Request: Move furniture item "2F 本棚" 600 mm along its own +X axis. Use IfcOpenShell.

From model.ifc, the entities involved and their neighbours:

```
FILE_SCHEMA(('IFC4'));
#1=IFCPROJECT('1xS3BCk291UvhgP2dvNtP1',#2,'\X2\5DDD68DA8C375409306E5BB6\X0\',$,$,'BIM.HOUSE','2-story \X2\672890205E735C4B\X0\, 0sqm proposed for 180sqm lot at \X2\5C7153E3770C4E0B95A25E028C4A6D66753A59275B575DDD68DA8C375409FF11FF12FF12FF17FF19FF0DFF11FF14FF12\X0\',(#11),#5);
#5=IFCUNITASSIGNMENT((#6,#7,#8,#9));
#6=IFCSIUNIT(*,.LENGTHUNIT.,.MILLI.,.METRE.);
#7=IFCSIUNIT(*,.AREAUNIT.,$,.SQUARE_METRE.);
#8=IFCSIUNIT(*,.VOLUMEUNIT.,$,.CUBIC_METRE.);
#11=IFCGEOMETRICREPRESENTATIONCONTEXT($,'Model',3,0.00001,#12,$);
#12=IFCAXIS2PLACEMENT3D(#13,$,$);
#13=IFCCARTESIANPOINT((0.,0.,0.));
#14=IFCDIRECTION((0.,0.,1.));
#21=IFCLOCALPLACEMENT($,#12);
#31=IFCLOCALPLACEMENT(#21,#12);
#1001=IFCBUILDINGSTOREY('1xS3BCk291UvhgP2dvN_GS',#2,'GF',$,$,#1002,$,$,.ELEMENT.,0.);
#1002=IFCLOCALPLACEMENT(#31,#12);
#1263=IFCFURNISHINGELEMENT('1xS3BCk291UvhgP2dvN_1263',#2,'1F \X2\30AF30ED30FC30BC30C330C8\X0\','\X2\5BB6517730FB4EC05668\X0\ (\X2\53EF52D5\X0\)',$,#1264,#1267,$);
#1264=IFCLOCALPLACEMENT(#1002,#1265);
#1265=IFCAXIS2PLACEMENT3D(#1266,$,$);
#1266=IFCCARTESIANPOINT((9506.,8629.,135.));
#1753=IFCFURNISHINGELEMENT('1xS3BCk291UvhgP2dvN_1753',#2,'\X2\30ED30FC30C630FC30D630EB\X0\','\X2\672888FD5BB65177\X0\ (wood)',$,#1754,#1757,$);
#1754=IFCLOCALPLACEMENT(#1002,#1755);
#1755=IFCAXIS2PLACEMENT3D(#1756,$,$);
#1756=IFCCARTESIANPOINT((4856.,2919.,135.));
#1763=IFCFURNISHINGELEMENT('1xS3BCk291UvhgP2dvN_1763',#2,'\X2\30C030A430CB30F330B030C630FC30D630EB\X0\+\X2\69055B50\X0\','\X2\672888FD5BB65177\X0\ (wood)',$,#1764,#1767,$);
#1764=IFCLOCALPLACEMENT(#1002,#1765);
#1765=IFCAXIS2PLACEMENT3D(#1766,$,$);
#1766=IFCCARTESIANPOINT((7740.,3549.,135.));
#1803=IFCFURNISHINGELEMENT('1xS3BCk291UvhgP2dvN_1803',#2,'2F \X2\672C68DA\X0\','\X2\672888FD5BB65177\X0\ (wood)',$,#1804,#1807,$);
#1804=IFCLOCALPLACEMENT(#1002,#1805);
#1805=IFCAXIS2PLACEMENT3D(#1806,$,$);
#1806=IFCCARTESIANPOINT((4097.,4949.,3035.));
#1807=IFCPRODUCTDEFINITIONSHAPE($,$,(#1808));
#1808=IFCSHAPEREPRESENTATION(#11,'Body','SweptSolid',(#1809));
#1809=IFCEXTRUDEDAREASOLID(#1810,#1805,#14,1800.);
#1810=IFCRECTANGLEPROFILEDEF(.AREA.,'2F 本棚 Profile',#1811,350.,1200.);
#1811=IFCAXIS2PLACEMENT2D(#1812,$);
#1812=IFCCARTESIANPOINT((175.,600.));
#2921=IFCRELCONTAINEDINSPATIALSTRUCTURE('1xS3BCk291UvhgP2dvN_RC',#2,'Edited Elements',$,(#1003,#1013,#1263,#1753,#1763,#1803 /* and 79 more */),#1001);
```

```python
import ifcopenshell
import ifcopenshell.api.geometry
import ifcopenshell.util.placement
import ifcopenshell.util.unit

model = ifcopenshell.open("model.ifc")
unit_scale = ifcopenshell.util.unit.calculate_unit_scale(model)

item = model.by_guid("1xS3BCk291UvhgP2dvN_1803")
matrix = ifcopenshell.util.placement.get_local_placement(item.ObjectPlacement)
matrix[:3, 3] += matrix[:3, 0] * 0.6 / unit_scale
ifcopenshell.api.geometry.edit_object_placement(model, product=item, matrix=matrix, is_si=False)

print(ifcopenshell.util.placement.get_local_placement(item.ObjectPlacement).round(3) + 0.0)

model.write("model_v2.ifc")
```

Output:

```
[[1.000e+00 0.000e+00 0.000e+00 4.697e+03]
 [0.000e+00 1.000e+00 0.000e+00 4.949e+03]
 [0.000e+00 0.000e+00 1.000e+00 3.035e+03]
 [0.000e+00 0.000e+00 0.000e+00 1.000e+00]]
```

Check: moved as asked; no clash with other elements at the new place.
